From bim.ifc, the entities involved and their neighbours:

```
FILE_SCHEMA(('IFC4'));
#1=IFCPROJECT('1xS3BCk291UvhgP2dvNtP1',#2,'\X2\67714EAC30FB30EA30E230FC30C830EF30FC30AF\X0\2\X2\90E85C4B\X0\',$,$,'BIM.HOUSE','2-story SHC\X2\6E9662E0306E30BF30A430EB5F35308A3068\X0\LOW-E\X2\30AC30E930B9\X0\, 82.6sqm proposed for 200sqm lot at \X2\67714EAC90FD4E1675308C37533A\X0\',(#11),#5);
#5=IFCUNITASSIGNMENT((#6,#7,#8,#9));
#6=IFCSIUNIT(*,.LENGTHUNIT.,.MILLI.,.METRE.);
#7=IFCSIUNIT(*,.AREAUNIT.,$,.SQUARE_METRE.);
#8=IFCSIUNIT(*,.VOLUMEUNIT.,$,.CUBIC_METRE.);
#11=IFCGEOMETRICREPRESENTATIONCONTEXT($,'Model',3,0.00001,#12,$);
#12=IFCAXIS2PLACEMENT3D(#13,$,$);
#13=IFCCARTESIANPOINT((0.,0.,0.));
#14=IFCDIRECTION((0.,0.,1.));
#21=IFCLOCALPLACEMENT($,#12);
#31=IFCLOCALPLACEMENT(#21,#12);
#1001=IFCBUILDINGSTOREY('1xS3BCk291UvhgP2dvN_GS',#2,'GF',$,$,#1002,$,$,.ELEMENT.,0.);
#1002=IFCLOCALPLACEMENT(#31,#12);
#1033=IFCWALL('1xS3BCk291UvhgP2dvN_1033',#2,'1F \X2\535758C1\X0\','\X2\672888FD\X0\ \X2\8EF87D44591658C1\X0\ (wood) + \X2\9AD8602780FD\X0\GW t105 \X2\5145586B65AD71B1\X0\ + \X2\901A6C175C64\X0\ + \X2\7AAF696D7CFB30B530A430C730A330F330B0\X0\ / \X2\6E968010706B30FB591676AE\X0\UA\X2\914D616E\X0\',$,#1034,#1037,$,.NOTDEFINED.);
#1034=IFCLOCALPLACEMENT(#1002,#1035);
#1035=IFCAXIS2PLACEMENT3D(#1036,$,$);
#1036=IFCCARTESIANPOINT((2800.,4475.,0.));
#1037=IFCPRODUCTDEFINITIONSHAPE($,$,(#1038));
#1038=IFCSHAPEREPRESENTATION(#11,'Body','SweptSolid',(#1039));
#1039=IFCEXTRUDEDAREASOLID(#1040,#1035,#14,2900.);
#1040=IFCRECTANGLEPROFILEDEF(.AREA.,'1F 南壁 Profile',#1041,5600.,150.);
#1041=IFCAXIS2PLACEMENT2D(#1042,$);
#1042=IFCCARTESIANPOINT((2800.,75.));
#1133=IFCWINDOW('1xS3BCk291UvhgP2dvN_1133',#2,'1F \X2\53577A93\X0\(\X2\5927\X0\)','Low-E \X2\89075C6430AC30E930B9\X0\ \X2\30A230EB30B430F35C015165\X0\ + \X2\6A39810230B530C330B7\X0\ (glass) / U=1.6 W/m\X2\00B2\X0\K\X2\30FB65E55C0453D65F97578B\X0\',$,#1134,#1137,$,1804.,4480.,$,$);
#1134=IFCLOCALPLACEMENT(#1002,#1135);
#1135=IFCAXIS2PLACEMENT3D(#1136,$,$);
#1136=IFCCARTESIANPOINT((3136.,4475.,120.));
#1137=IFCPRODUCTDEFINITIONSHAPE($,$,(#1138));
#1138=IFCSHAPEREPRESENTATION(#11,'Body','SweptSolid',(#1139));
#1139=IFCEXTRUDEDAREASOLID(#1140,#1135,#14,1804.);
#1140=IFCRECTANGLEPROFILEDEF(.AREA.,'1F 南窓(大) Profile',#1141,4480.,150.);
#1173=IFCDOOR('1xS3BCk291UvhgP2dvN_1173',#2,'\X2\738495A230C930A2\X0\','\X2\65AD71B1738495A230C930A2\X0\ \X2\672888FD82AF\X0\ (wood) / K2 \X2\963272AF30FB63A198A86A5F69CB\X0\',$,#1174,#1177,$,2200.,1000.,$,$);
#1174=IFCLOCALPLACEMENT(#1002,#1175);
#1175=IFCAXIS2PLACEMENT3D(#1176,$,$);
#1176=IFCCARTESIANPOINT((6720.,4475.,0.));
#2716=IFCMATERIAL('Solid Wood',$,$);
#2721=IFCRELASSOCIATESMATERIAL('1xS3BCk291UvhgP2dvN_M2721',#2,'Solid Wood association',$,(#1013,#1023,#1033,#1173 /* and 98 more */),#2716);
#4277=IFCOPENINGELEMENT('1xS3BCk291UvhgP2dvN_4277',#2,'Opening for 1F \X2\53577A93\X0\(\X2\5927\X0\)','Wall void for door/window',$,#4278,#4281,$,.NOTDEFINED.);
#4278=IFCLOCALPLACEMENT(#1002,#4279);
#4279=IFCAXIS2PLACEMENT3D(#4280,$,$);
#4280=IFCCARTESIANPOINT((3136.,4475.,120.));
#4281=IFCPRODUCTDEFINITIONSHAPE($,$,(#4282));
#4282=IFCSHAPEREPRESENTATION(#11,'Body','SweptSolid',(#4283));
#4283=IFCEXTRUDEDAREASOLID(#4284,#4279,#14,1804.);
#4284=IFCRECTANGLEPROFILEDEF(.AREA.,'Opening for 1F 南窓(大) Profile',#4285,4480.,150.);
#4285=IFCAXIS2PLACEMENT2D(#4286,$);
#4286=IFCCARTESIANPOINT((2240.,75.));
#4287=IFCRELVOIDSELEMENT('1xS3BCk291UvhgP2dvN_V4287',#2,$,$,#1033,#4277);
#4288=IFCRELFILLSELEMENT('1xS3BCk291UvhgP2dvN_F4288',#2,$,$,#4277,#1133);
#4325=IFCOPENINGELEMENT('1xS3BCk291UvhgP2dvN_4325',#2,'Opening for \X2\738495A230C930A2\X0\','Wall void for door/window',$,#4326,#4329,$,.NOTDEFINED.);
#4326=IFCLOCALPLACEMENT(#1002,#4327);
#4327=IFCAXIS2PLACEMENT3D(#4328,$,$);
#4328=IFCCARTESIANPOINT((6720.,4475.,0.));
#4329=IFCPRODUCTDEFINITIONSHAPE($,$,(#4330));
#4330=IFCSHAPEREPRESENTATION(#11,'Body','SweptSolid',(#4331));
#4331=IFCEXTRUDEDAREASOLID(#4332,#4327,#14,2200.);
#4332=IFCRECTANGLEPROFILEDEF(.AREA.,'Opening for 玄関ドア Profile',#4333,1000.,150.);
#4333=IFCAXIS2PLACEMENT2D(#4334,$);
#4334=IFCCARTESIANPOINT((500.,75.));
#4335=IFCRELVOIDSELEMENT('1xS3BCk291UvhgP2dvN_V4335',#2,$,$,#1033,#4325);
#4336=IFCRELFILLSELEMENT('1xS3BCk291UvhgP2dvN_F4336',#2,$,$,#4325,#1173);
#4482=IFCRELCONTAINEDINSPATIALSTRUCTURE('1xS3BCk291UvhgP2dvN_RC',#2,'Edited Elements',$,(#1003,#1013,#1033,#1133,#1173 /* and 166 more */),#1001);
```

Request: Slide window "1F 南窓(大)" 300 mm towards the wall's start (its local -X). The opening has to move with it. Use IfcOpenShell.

```python
import ifcopenshell
import ifcopenshell.api.geometry
import ifcopenshell.util.placement

model = ifcopenshell.open("bim.ifc")

window = model.by_id(1133)
opening = window.FillsVoids[0].RelatingOpeningElement
wall = opening.VoidsElements[0].RelatingBuildingElement

wall_matrix = ifcopenshell.util.placement.get_local_placement(wall.ObjectPlacement)
shift = wall_matrix[:3, 0] * -300.0
before = ifcopenshell.util.placement.get_local_placement(window.ObjectPlacement)[:3, 3].copy()

# The window is not placed relative to its opening, so move both.
for product in (opening, window):
    matrix = ifcopenshell.util.placement.get_local_placement(product.ObjectPlacement)
    matrix[:3, 3] += shift
    ifcopenshell.api.geometry.edit_object_placement(model, product=product, matrix=matrix, is_si=False)

after = ifcopenshell.util.placement.get_local_placement(window.ObjectPlacement)[:3, 3]
print("window moved by", (after - before).round(3) + 0.0)

model.write("bim_v2.ifc")
```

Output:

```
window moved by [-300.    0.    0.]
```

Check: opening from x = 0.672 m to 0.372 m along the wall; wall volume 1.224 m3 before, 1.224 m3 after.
